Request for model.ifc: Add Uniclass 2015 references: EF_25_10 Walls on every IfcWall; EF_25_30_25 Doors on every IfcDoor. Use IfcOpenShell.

First a look at what the model holds.

```python
import ifcopenshell

model = ifcopenshell.open("model.ifc")
print(model.schema)
print("classifications:", [c.Name for c in model.by_type("IfcClassification")])
for ifc_class in ("IfcDoor", "IfcRoof", "IfcStair", "IfcWall", "IfcWindow"):
    print(ifc_class, len(model.by_type(ifc_class)))
```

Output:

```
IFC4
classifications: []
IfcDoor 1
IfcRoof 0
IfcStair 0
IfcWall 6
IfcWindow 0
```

```python
import ifcopenshell
import ifcopenshell.api.classification

model = ifcopenshell.open("model.ifc")

system = ifcopenshell.api.classification.add_classification(model, classification="Uniclass 2015")

codes = {
    "IfcWall": ("EF_25_10", "Walls"),
    "IfcDoor": ("EF_25_30_25", "Doors"),
}
for ifc_class, (code, name) in codes.items():
    products = model.by_type(ifc_class)
    ifcopenshell.api.classification.add_reference(
        model, products=products, classification=system, identification=code, name=name
    )
    print(code, len(products))

model.write("model_v2.ifc")
```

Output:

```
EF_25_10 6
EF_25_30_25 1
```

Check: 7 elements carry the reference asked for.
